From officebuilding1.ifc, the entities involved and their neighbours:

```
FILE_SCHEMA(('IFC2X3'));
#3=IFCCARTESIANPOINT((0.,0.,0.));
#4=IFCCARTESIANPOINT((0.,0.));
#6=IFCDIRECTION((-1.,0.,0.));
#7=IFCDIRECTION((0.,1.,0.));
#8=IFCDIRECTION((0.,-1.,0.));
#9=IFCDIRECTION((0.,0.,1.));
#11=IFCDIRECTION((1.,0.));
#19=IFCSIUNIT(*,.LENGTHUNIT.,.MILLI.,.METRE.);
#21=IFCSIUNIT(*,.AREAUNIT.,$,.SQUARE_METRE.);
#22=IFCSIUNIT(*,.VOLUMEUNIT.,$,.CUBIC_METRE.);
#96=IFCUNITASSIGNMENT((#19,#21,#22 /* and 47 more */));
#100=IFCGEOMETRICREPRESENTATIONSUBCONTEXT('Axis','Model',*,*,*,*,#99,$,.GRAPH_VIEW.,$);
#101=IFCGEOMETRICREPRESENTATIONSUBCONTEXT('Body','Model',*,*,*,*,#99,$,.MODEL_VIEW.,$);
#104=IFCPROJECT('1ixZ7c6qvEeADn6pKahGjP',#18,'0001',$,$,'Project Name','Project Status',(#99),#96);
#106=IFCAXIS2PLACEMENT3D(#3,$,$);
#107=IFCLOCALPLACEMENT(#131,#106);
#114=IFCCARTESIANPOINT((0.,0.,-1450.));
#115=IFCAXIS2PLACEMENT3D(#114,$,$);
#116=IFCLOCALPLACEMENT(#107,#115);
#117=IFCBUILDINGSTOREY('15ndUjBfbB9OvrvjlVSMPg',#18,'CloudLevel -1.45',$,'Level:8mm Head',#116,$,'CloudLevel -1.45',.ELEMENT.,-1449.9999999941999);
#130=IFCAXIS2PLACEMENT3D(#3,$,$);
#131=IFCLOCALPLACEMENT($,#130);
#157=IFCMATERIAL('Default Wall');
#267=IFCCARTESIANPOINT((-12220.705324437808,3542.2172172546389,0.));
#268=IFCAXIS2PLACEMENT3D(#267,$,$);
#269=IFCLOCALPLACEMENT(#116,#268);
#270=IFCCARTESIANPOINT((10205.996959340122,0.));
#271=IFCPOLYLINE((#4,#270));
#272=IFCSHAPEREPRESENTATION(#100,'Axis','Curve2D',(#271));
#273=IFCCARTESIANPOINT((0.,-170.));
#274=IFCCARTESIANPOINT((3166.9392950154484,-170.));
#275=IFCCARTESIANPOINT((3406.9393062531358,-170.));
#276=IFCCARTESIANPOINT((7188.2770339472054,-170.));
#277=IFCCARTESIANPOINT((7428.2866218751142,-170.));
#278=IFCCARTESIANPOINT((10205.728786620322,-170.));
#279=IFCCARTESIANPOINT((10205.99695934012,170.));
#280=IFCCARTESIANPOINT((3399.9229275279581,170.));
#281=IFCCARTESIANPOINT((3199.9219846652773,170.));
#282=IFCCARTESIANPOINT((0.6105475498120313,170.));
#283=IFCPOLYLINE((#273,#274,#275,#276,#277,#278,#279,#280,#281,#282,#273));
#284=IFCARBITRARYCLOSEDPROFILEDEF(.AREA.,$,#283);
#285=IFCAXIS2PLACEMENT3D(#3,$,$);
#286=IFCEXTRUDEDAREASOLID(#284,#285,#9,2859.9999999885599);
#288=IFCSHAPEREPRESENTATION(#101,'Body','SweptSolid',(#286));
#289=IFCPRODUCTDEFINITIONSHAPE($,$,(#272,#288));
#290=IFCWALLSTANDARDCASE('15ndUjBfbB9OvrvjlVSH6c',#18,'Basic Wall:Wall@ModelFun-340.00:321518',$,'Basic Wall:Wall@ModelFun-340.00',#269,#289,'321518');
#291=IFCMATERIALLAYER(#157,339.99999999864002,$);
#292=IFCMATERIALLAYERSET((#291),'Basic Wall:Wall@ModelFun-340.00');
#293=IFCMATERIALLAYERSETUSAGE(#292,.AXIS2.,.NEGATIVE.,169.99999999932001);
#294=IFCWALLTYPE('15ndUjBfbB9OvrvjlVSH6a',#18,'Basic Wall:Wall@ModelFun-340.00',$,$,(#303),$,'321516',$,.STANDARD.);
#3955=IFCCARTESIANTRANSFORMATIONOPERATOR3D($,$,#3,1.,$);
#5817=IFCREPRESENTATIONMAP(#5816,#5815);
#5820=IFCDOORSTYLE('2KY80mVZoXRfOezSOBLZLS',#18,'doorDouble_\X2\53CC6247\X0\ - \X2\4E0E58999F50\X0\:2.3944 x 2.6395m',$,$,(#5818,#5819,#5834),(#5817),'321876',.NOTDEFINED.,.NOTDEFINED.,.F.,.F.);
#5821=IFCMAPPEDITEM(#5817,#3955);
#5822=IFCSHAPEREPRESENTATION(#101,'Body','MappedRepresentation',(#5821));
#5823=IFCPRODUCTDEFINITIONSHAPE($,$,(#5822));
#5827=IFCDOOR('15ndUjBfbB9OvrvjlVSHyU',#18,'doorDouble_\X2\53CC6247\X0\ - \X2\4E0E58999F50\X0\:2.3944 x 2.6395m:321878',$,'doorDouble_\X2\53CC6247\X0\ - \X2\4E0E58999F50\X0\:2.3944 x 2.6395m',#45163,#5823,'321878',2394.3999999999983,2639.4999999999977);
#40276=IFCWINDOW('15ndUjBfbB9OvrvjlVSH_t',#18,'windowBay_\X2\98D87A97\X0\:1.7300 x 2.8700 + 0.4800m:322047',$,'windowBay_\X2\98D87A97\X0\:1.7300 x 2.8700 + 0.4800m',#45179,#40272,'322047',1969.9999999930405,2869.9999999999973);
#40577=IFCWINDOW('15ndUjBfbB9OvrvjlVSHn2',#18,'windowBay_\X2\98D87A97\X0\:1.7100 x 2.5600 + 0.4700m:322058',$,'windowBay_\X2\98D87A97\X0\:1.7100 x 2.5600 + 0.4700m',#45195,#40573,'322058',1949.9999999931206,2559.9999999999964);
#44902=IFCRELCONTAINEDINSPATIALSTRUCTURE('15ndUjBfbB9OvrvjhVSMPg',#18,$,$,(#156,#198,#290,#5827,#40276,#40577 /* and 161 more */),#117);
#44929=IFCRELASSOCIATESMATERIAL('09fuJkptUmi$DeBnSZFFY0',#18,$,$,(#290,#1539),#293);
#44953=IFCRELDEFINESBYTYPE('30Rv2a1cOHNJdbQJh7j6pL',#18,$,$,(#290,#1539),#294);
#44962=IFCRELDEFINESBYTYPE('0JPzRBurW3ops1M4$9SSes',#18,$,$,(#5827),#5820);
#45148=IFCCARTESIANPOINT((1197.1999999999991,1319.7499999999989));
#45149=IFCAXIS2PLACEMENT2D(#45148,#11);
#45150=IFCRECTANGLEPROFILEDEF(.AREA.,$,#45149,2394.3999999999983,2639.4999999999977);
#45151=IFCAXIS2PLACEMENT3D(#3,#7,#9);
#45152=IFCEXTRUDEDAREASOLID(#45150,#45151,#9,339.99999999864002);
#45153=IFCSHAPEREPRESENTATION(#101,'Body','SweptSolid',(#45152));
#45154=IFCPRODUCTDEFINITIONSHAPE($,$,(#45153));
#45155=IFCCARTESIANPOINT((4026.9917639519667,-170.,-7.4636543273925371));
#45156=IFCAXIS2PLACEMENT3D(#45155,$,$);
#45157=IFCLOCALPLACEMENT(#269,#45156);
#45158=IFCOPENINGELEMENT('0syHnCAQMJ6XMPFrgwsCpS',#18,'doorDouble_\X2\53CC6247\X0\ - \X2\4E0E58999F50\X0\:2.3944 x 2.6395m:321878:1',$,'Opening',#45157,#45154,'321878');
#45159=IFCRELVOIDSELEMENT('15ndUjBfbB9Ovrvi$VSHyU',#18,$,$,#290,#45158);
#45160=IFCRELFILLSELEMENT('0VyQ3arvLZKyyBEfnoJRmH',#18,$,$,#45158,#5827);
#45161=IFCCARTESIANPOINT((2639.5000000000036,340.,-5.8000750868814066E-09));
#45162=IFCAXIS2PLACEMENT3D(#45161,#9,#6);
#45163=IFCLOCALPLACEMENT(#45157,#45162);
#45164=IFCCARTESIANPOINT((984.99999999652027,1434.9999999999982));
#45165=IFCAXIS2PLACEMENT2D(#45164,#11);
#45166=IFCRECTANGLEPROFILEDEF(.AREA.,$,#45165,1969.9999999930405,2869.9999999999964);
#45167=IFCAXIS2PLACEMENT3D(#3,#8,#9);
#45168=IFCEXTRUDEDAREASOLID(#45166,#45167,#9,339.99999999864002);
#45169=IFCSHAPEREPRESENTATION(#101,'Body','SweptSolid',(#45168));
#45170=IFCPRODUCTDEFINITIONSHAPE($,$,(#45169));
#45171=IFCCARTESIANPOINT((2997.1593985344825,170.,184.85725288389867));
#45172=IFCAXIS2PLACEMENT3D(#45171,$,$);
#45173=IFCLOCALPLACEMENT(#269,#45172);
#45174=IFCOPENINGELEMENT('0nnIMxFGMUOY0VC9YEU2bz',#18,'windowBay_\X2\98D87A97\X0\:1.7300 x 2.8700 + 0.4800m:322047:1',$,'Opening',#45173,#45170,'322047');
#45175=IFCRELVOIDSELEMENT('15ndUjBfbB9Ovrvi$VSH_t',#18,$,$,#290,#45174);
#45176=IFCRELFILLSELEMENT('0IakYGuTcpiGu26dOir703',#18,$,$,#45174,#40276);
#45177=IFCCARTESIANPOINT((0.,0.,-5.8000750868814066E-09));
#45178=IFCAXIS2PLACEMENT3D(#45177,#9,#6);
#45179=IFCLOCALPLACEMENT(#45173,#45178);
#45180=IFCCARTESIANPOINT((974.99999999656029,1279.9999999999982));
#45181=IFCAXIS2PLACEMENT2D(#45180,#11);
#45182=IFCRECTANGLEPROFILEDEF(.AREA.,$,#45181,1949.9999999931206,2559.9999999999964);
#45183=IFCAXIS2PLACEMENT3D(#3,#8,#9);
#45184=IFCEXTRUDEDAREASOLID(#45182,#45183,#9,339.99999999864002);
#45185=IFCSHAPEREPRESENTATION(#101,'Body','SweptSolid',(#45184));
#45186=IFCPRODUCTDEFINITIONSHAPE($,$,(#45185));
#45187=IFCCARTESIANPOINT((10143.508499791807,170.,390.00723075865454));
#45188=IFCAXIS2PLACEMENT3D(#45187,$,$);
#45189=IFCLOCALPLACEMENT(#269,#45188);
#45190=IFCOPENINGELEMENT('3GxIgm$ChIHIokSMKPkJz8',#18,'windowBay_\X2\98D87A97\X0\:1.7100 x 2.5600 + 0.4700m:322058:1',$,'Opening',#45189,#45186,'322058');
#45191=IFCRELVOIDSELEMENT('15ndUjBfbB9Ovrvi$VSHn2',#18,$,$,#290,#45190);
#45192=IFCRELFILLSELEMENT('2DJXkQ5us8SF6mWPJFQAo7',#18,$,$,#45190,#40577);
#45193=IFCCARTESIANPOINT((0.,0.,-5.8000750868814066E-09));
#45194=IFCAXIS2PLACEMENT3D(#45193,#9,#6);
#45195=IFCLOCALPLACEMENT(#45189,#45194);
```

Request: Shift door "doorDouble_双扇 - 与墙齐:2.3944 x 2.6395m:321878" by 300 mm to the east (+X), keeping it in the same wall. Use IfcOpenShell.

```python
import ifcopenshell
import ifcopenshell.api.geometry
import ifcopenshell.util.placement

model = ifcopenshell.open("officebuilding1.ifc")

door = model.by_guid("15ndUjBfbB9OvrvjlVSHyU")
opening = door.FillsVoids[0].RelatingOpeningElement
wall = opening.VoidsElements[0].RelatingBuildingElement

wall_matrix = ifcopenshell.util.placement.get_local_placement(wall.ObjectPlacement)
shift = wall_matrix[:3, 0] * 300.0
before = ifcopenshell.util.placement.get_local_placement(door.ObjectPlacement)[:3, 3].copy()

# The door is placed relative to its opening, so it follows when the opening moves.
matrix = ifcopenshell.util.placement.get_local_placement(opening.ObjectPlacement)
matrix[:3, 3] += shift
ifcopenshell.api.geometry.edit_object_placement(
    model, product=opening, matrix=matrix, is_si=False, should_transform_children=True
)

after = ifcopenshell.util.placement.get_local_placement(door.ObjectPlacement)[:3, 3]
print("door moved by", (after - before).round(3) + 0.0)

model.write("officebuilding1_rev.ifc")
```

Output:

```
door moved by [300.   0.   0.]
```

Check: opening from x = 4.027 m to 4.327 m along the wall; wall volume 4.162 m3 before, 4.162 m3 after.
